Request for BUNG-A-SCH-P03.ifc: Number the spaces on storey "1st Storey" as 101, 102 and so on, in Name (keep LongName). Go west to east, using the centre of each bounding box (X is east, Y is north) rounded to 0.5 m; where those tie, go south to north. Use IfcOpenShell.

First a look at what the model holds.

```python
import ifcopenshell
import ifcopenshell.util.element
import ifcopenshell.util.placement

model = ifcopenshell.open("BUNG-A-SCH-P03.ifc")
print(model.schema)
storey = next(s for s in model.by_type("IfcBuildingStorey") if s.Name == "1st Storey")
spaces = [e for e in ifcopenshell.util.element.get_decomposition(storey) if e.is_a("IfcSpace")]
for e in sorted(spaces, key=lambda e: e.id()):
    origin = ifcopenshell.util.placement.get_local_placement(e.ObjectPlacement)[:3, 3]
    print(e.id(), e.Name, e.LongName, origin.round(2) + 0.0, sep=" | ")
```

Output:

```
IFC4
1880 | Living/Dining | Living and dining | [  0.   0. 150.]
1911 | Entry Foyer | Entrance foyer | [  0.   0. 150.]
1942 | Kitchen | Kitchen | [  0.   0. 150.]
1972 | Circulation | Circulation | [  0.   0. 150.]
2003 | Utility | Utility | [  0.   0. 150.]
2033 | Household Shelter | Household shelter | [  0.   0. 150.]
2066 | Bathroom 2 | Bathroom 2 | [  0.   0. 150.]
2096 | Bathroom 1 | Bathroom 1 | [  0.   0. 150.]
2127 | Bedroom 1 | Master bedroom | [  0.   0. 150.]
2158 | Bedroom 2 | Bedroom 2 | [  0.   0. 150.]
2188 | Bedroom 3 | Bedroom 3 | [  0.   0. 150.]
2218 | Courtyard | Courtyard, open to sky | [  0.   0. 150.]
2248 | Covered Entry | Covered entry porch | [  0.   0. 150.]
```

```python
import ifcopenshell
import ifcopenshell.geom
import ifcopenshell.util.element
import ifcopenshell.util.shape

model = ifcopenshell.open("BUNG-A-SCH-P03.ifc")
settings = ifcopenshell.geom.settings()
settings.set("use-world-coords", True)


def centre(element):
    shape = ifcopenshell.geom.create_shape(settings, element)
    return ifcopenshell.util.shape.get_bbox_centroid(shape.geometry)


storey = next(s for s in model.by_type("IfcBuildingStorey") if s.Name == "1st Storey")
spaces = [e for e in ifcopenshell.util.element.get_decomposition(storey) if e.is_a("IfcSpace")]

# Insertion points can sit at a corner or the storey origin, so sort by the geometry (in metres).
centres = {e: centre(e) for e in spaces}
spaces.sort(key=lambda e: (round(centres[e][0] / 0.5), centres[e][1]))

for i, e in enumerate(spaces, start=1):
    number = f"1{i:02d}"
    e.Name = number
    print(e.id(), number)

model.write("BUNG-A-SCH-P03_v2.ifc")
```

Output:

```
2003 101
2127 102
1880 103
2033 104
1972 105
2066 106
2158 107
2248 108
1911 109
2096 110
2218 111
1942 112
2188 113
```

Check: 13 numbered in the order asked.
